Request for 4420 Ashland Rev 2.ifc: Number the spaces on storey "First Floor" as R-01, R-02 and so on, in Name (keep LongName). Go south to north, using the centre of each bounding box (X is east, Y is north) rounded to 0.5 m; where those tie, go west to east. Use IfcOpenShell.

First a look at what the model holds.

```python
import ifcopenshell
import ifcopenshell.util.element
import ifcopenshell.util.placement

model = ifcopenshell.open("4420 Ashland Rev 2.ifc")
print(model.schema)
storey = next(s for s in model.by_type("IfcBuildingStorey") if s.Name == "First Floor")
spaces = [e for e in ifcopenshell.util.element.get_decomposition(storey) if e.is_a("IfcSpace")]
for e in sorted(spaces, key=lambda e: e.id()):
    origin = ifcopenshell.util.placement.get_local_placement(e.ObjectPlacement)[:3, 3]
    print(e.id(), e.Name, e.LongName, origin.round(2) + 0.0, sep=" | ")
```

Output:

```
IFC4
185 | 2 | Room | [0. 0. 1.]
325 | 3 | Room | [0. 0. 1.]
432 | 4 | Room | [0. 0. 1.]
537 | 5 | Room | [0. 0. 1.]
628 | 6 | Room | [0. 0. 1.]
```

```python
import ifcopenshell
import ifcopenshell.geom
import ifcopenshell.util.element
import ifcopenshell.util.shape

model = ifcopenshell.open("4420 Ashland Rev 2.ifc")
settings = ifcopenshell.geom.settings()
settings.set("use-world-coords", True)


def centre(element):
    shape = ifcopenshell.geom.create_shape(settings, element)
    return ifcopenshell.util.shape.get_bbox_centroid(shape.geometry)


storey = next(s for s in model.by_type("IfcBuildingStorey") if s.Name == "First Floor")
spaces = [e for e in ifcopenshell.util.element.get_decomposition(storey) if e.is_a("IfcSpace")]

# Insertion points can sit at a corner or the storey origin, so sort by the geometry (in metres).
centres = {e: centre(e) for e in spaces}
spaces.sort(key=lambda e: (round(centres[e][1] / 0.5), centres[e][0]))

for i, e in enumerate(spaces, start=1):
    number = f"R-{i:02d}"
    e.Name = number
    print(e.id(), number)

model.write("4420 Ashland Rev 2-out.ifc")
```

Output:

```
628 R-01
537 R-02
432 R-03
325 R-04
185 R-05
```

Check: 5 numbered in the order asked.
